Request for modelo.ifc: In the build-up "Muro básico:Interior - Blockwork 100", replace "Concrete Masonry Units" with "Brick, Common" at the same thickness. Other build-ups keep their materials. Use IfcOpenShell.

First a look at what the model holds.

```python
import ifcopenshell
import ifcopenshell.util.element

model = ifcopenshell.open("modelo.ifc")
print(model.schema)
for layer_set in model.by_type("IfcMaterialLayerSet"):
    if layer_set.LayerSetName == "Muro básico:Interior - Blockwork 100":
        for layer in layer_set.MaterialLayers:
            print(layer.id(), layer.Material and layer.Material.Name, layer.LayerThickness, sep=" | ")
        print(len(ifcopenshell.util.element.get_elements_by_material(model, layer_set)), "elements and types use it")
print(sorted(m.Name for m in model.by_type("IfcMaterial") if m.Name)[:60])
```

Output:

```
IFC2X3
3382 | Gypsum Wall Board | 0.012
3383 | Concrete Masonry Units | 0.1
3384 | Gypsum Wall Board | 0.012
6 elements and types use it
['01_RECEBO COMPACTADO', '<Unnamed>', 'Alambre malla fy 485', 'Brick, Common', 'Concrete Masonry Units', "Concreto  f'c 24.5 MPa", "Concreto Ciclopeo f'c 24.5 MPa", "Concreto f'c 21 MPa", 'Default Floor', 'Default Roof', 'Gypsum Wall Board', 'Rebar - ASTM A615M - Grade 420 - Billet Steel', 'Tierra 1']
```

```python
import ifcopenshell
import ifcopenshell.api.material

model = ifcopenshell.open("modelo.ifc")

layer_set = next(s for s in model.by_type("IfcMaterialLayerSet") if s.LayerSetName == "Muro básico:Interior - Blockwork 100")
layer = next(l for l in layer_set.MaterialLayers if l.Material and l.Material.Name == "Concrete Masonry Units")
material = next(m for m in model.by_type("IfcMaterial") if m.Name == "Brick, Common")

# Point this one layer at the other material; renaming the old one would change it everywhere.
ifcopenshell.api.material.edit_layer(model, layer=layer, attributes={}, material=material)

print([l.Material.Name if l.Material else None for l in layer_set.MaterialLayers])

model.write("modelo_edited.ifc")
```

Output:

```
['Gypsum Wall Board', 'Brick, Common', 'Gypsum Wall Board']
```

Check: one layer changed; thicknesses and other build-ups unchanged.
